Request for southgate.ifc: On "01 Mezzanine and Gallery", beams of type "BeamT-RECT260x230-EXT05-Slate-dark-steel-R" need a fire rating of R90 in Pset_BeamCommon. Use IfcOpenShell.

First a look at what the model holds.

```python
import ifcopenshell
import ifcopenshell.util.element

model = ifcopenshell.open("southgate.ifc")
print(model.schema)
storey = next(s for s in model.by_type("IfcBuildingStorey") if s.Name == "01 Mezzanine and Gallery")
beams = [e for e in ifcopenshell.util.element.get_decomposition(storey) if e.is_a("IfcBeam")]
seen = {}
for e in beams:
    element_type = ifcopenshell.util.element.get_type(e)
    key = (element_type.Name if element_type != e and element_type else None, ifcopenshell.util.element.get_pset(e, "Pset_BeamCommon", "FireRating"))
    seen[key] = seen.get(key, 0) + 1
for (name, value), count in sorted(seen.items(), key=str):
    print(count, "x", name, "|", value)
```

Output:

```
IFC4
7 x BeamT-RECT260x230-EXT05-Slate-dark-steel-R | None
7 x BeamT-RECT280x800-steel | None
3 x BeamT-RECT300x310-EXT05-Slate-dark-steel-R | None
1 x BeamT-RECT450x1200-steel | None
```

```python
import ifcopenshell
import ifcopenshell.api.pset
import ifcopenshell.util.element

model = ifcopenshell.open("southgate.ifc")

storey = next(s for s in model.by_type("IfcBuildingStorey") if s.Name == "01 Mezzanine and Gallery")
beams = [e for e in ifcopenshell.util.element.get_decomposition(storey) if e.is_a("IfcBeam")]

count = 0
for e in beams:
    element_type = ifcopenshell.util.element.get_type(e)
    if element_type in (None, e) or element_type.Name != "BeamT-RECT260x230-EXT05-Slate-dark-steel-R":
        continue
    # add_pset returns the element's existing set when there is one.
    pset = ifcopenshell.api.pset.add_pset(model, product=e, name="Pset_BeamCommon")
    ifcopenshell.api.pset.edit_pset(model, pset=pset, properties={"FireRating": "R90"})
    count += 1

print(count, "beams updated")

model.write("southgate_rev.ifc")
```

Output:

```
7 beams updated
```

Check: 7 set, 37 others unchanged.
